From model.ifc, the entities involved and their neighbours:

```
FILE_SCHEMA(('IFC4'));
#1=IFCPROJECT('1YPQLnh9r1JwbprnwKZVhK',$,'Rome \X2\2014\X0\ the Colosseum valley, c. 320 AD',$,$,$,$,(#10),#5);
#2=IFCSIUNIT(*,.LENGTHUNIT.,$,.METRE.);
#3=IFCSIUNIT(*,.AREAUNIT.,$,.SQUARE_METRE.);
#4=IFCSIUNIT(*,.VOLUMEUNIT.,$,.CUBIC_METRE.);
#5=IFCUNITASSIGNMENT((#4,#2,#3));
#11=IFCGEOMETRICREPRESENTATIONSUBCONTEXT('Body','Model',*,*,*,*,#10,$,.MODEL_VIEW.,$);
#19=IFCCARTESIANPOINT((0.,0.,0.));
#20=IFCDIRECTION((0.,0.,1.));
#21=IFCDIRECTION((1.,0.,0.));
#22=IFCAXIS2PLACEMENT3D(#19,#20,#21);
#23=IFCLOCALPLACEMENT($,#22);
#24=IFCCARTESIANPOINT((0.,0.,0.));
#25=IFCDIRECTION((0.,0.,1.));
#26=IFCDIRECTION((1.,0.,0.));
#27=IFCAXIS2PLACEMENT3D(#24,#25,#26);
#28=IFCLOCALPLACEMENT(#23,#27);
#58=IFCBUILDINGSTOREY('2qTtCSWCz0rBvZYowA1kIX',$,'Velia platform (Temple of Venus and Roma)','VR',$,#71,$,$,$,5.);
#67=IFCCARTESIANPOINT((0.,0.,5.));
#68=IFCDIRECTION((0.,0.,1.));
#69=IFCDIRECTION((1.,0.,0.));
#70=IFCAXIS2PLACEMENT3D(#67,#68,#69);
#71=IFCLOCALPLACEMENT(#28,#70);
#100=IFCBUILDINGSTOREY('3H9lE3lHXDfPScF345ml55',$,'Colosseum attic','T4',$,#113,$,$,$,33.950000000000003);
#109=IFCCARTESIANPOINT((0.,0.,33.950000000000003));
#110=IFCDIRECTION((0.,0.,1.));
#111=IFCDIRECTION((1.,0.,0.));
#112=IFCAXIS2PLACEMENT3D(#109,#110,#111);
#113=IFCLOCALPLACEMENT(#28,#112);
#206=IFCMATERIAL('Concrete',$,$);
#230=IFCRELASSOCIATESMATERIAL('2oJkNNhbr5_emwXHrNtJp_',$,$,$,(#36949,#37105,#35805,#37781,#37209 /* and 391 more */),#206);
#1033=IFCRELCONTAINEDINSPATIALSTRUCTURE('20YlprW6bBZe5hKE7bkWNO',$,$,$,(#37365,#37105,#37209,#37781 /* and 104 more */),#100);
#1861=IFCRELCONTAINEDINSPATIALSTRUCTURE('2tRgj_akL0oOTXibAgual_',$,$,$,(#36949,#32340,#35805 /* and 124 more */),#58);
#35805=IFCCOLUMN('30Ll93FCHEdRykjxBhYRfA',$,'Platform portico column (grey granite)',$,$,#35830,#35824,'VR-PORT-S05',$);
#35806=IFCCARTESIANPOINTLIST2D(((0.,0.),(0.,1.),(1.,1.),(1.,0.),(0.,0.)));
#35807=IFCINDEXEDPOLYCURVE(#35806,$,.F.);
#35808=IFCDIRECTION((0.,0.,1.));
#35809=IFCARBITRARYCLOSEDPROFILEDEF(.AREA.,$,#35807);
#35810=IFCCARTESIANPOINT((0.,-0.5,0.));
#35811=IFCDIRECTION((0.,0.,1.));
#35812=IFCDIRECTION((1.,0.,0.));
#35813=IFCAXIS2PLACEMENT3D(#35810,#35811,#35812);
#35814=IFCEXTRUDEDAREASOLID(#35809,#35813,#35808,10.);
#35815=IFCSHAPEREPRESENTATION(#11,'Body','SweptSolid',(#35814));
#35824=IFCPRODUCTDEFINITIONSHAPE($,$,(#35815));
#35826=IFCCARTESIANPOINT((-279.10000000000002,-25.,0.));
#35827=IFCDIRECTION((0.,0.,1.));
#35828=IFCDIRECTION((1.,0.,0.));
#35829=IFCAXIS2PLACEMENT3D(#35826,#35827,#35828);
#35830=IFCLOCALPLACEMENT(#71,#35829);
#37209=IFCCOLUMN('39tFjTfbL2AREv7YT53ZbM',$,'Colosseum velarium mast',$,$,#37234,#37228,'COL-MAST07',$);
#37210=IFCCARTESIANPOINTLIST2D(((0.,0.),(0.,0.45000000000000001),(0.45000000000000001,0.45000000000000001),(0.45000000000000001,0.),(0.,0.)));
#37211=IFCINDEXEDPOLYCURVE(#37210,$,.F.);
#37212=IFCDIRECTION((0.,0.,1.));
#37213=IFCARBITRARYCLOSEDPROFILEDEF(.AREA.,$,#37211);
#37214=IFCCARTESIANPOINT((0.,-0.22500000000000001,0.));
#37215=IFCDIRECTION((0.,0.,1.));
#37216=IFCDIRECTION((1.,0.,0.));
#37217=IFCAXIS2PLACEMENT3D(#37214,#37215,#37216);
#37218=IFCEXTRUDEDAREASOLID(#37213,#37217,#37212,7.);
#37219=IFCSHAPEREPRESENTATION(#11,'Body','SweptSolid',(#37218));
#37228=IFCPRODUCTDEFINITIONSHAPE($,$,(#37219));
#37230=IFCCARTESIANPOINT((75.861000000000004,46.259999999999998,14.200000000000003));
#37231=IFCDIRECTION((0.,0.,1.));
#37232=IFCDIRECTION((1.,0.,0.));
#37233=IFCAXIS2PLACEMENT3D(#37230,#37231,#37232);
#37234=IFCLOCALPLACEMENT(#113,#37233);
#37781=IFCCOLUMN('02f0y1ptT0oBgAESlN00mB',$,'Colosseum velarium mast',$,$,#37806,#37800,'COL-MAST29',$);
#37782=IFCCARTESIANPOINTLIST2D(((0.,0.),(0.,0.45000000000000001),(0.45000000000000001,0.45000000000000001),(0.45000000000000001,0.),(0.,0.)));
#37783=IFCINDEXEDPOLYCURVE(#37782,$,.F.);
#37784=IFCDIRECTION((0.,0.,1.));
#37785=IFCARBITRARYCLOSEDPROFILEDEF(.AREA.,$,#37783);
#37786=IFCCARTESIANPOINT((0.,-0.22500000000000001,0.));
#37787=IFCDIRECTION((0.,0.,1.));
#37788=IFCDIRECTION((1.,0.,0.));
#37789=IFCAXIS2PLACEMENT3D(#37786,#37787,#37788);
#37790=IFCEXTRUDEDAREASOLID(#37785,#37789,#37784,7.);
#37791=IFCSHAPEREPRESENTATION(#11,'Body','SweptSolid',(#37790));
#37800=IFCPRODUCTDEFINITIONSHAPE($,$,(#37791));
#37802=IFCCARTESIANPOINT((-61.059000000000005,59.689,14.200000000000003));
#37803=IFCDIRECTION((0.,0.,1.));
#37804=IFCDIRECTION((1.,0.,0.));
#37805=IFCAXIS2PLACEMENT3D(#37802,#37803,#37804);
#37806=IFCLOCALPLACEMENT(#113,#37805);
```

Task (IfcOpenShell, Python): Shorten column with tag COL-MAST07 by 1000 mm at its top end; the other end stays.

```python
import ifcopenshell
import ifcopenshell.util.representation

model = ifcopenshell.open("model.ifc")

member = model.by_guid("39tFjTfbL2AREv7YT53ZbM")
change = -1.0

# The extrusion runs towards the end named, so only its depth changes.
body = ifcopenshell.util.representation.get_representation(member, "Model", "Body")
solid = body.Items[0]
old_length = solid.Depth
solid.Depth += change

print(f"length {old_length:g} -> {solid.Depth:g}")

model.write("model_v2.ifc")
```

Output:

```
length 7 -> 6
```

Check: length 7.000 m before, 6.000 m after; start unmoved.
